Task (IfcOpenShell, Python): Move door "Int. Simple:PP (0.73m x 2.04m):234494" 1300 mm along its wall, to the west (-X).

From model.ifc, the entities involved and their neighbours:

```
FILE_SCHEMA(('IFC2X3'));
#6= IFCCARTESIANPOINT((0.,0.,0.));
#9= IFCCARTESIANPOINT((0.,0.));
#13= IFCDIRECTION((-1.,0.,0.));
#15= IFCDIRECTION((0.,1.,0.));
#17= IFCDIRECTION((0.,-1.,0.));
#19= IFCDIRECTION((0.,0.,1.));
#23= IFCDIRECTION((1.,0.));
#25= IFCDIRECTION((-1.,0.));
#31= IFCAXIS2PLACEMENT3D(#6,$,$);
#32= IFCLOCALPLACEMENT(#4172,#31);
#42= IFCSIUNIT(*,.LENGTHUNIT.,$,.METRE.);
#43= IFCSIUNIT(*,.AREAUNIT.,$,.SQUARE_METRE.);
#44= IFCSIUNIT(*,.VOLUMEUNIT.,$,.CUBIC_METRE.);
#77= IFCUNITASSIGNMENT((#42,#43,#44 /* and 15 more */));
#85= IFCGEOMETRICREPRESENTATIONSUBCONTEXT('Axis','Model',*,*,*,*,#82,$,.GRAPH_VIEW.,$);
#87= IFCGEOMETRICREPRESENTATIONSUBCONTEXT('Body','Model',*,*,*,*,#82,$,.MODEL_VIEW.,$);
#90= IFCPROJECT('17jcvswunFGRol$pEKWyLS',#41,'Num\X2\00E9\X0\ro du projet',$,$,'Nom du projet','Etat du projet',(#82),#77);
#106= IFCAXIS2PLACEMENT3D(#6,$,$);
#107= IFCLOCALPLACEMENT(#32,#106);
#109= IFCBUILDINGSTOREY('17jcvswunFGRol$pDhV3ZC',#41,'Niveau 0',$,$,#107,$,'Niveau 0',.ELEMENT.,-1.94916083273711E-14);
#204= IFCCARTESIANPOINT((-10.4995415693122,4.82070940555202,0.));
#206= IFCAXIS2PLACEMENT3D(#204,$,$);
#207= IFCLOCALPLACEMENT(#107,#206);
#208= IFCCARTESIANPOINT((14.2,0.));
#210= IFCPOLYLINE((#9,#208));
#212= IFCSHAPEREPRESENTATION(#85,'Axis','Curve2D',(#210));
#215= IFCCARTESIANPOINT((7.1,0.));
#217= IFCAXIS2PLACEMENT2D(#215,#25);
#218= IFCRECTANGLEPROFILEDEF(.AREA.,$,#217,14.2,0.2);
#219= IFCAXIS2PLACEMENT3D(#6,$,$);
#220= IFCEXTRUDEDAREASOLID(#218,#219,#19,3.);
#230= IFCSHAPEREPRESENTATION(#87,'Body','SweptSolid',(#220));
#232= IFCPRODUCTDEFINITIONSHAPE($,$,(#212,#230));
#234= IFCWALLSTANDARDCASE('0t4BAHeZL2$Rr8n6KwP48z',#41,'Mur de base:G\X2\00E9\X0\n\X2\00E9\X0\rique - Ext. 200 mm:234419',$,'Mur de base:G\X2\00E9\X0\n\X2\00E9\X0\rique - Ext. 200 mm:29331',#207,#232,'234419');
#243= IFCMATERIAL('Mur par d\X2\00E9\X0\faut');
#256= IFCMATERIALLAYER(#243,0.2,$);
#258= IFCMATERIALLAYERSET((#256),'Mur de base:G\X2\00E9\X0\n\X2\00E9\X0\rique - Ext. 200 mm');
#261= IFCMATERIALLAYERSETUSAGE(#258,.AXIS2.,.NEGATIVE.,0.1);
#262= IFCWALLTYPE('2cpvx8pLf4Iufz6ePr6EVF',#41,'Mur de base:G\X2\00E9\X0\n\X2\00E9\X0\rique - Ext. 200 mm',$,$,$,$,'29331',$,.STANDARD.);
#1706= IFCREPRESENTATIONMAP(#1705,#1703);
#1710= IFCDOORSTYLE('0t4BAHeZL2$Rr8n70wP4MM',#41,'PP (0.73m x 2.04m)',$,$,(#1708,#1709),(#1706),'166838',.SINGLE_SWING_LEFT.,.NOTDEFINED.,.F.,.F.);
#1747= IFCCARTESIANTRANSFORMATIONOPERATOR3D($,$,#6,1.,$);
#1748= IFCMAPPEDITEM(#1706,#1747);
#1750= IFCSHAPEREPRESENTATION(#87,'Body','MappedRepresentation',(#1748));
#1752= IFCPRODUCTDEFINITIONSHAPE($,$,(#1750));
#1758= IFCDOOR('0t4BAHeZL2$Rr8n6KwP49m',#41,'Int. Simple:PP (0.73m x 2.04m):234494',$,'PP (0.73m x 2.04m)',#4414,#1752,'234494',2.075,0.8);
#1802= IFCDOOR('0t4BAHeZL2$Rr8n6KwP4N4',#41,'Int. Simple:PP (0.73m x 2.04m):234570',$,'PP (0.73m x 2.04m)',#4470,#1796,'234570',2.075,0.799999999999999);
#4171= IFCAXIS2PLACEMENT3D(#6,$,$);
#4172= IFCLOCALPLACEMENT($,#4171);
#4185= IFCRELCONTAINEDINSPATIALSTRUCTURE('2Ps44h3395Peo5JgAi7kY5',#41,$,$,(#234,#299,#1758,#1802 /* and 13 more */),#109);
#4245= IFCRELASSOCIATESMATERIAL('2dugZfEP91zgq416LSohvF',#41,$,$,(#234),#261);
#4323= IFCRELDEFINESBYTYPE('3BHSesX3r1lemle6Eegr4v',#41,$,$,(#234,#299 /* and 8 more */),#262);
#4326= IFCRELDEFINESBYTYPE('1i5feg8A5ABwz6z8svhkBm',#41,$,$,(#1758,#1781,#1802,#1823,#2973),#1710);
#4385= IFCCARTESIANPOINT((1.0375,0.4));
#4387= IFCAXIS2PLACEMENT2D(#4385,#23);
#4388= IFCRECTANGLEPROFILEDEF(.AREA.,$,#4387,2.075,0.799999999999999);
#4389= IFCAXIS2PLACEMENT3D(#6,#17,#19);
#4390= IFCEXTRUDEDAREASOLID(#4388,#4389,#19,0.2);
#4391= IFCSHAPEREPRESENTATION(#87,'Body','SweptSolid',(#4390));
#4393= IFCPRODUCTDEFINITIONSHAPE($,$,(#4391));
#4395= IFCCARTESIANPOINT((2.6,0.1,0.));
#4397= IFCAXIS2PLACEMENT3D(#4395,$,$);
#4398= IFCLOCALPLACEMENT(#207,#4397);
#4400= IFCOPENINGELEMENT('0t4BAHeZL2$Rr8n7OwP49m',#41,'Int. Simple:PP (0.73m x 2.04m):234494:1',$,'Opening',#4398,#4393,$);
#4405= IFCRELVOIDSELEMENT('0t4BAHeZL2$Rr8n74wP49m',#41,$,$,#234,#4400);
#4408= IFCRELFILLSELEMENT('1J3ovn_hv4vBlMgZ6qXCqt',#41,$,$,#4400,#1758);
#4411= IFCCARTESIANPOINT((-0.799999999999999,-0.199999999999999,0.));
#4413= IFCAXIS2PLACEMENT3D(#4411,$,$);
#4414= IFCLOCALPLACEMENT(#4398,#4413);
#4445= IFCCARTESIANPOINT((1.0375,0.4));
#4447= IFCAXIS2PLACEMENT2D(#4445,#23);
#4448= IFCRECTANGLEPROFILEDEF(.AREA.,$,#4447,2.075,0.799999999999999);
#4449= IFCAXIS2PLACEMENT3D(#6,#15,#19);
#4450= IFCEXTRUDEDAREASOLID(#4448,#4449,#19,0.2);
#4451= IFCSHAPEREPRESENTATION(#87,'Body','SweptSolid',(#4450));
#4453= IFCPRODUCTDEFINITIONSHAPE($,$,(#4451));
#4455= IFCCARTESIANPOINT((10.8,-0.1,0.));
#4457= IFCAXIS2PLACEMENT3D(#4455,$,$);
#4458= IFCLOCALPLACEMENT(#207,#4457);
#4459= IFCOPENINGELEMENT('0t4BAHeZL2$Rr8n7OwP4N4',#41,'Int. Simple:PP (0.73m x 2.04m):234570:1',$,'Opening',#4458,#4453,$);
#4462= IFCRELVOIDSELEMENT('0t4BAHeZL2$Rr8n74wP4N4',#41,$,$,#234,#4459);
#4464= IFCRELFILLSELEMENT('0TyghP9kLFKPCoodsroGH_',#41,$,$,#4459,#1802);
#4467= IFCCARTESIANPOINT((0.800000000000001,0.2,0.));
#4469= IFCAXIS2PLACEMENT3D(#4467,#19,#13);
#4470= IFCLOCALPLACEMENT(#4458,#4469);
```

```python
import ifcopenshell
import ifcopenshell.api.geometry
import ifcopenshell.util.placement
import ifcopenshell.util.unit

model = ifcopenshell.open("model.ifc")
unit_scale = ifcopenshell.util.unit.calculate_unit_scale(model)

door = model.by_guid("0t4BAHeZL2$Rr8n6KwP49m")
opening = door.FillsVoids[0].RelatingOpeningElement
wall = opening.VoidsElements[0].RelatingBuildingElement

wall_matrix = ifcopenshell.util.placement.get_local_placement(wall.ObjectPlacement)
shift = wall_matrix[:3, 0] * -1.3 / unit_scale
before = ifcopenshell.util.placement.get_local_placement(door.ObjectPlacement)[:3, 3].copy()

# The door is placed relative to its opening, so it follows when the opening moves.
matrix = ifcopenshell.util.placement.get_local_placement(opening.ObjectPlacement)
matrix[:3, 3] += shift
ifcopenshell.api.geometry.edit_object_placement(
    model, product=opening, matrix=matrix, is_si=False, should_transform_children=True
)

after = ifcopenshell.util.placement.get_local_placement(door.ObjectPlacement)[:3, 3]
print("door moved by", (after - before).round(3) + 0.0)

model.write("model_v2.ifc")
```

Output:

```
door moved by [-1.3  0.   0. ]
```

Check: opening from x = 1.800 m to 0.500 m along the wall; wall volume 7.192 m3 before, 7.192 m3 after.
